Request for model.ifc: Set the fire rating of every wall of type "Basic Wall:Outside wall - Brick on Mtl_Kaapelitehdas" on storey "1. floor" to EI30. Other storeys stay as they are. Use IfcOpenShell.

First a look at what the model holds.

```python
import ifcopenshell
import ifcopenshell.util.element

model = ifcopenshell.open("model.ifc")
print(model.schema)
storey = next(s for s in model.by_type("IfcBuildingStorey") if s.Name == "1. floor")
walls = [e for e in ifcopenshell.util.element.get_decomposition(storey) if e.is_a("IfcWall")]
seen = {}
for e in walls:
    element_type = ifcopenshell.util.element.get_type(e)
    key = (element_type.Name if element_type != e and element_type else None, ifcopenshell.util.element.get_pset(e, "Pset_WallCommon", "FireRating"))
    seen[key] = seen.get(key, 0) + 1
for (name, value), count in sorted(seen.items(), key=str):
    print(count, "x", name, "|", value)
```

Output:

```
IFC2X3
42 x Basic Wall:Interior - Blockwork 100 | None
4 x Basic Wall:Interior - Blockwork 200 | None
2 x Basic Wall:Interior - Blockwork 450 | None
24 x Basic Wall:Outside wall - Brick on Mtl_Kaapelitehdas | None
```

```python
import ifcopenshell
import ifcopenshell.api.pset
import ifcopenshell.util.element

model = ifcopenshell.open("model.ifc")

storey = next(s for s in model.by_type("IfcBuildingStorey") if s.Name == "1. floor")
walls = [e for e in ifcopenshell.util.element.get_decomposition(storey) if e.is_a("IfcWall")]

count = 0
for e in walls:
    element_type = ifcopenshell.util.element.get_type(e)
    if element_type in (None, e) or element_type.Name != "Basic Wall:Outside wall - Brick on Mtl_Kaapelitehdas":
        continue
    # add_pset returns the element's existing set when there is one.
    pset = ifcopenshell.api.pset.add_pset(model, product=e, name="Pset_WallCommon")
    ifcopenshell.api.pset.edit_pset(model, pset=pset, properties={"FireRating": "EI30"})
    count += 1

print(count, "walls updated")

model.write("model_edited.ifc")
```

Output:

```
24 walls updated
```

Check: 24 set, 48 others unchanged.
